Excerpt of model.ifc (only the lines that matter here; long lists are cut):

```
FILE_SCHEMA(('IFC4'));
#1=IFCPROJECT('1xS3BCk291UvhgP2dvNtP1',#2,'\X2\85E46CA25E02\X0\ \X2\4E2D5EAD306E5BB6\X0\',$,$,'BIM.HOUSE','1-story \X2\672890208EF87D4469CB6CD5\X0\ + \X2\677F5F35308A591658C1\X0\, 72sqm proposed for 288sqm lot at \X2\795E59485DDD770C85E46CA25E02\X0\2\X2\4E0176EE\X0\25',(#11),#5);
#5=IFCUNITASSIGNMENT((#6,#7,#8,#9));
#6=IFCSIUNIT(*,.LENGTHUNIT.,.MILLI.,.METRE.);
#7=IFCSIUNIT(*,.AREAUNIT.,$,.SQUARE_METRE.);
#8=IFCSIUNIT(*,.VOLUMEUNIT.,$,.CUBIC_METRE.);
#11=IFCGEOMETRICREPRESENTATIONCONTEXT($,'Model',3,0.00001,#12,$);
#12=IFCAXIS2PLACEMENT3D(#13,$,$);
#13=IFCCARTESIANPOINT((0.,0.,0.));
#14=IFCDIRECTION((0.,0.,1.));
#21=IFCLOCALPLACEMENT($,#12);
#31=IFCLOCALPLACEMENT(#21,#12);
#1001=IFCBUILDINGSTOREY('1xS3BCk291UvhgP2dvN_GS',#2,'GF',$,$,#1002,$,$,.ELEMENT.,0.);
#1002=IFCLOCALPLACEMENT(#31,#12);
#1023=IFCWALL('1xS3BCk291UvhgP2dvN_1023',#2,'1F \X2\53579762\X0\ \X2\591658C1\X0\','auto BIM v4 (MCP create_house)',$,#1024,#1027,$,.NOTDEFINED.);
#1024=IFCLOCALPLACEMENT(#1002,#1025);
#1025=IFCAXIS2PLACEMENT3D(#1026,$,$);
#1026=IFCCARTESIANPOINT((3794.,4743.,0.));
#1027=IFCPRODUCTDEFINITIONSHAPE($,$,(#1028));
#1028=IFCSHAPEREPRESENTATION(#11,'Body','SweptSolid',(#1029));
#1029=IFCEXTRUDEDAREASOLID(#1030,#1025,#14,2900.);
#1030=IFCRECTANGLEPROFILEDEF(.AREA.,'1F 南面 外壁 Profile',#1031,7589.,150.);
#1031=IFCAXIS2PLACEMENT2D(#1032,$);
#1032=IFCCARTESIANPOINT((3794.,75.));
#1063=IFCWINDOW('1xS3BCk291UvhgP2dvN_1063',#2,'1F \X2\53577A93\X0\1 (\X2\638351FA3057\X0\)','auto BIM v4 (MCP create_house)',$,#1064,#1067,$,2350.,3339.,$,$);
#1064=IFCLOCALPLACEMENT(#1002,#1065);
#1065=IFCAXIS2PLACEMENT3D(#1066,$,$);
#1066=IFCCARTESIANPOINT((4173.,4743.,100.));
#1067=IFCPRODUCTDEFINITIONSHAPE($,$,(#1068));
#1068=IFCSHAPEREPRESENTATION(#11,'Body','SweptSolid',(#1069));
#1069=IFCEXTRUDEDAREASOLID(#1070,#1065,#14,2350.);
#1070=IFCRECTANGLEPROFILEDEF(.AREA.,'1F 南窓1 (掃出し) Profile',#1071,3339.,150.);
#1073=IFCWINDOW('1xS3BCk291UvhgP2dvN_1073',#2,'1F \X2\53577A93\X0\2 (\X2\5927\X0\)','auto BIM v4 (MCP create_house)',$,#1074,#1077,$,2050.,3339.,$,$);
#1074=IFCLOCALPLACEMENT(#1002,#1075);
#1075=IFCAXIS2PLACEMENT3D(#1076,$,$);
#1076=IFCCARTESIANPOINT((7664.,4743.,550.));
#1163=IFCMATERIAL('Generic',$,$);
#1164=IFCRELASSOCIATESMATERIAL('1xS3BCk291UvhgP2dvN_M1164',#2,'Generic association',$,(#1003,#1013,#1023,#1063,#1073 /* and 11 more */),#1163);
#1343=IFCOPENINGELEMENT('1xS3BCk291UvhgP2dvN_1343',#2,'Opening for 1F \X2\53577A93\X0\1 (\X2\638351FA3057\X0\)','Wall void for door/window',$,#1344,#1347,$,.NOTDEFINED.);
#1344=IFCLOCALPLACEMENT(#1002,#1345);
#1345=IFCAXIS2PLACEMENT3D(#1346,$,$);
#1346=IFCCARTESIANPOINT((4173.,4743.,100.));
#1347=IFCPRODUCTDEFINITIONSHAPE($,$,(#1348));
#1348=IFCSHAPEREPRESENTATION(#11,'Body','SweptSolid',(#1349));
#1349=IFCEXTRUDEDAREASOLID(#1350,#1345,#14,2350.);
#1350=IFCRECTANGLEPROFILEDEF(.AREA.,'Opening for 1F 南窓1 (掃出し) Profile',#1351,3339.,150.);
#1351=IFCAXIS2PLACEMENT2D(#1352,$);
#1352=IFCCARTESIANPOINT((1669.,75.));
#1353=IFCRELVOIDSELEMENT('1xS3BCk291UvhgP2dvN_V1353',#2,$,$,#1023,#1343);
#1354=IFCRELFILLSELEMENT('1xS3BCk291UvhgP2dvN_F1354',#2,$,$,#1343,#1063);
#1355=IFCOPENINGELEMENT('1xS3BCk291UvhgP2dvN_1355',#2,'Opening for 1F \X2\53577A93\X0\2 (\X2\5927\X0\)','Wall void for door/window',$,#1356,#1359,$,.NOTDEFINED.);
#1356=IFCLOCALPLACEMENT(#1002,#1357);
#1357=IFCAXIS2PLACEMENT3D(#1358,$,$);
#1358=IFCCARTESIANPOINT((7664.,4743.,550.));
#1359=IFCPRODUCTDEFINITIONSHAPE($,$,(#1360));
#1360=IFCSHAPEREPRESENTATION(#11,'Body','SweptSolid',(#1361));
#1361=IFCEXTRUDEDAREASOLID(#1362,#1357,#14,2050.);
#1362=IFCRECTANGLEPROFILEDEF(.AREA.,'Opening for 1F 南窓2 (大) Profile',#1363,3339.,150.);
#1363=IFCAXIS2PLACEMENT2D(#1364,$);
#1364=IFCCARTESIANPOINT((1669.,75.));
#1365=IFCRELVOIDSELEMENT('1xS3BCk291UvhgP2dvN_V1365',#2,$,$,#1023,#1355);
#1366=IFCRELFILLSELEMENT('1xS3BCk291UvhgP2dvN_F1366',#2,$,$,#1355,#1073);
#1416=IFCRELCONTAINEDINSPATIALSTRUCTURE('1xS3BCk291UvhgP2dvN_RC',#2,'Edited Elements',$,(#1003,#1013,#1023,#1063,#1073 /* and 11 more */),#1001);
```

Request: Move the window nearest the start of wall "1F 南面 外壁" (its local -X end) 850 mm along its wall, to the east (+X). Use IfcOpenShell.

```python
import ifcopenshell
import ifcopenshell.api.geometry
import ifcopenshell.util.placement
import ifcopenshell.util.unit

model = ifcopenshell.open("model.ifc")
unit_scale = ifcopenshell.util.unit.calculate_unit_scale(model)

window = model.by_guid("1xS3BCk291UvhgP2dvN_1063")
opening = window.FillsVoids[0].RelatingOpeningElement
wall = opening.VoidsElements[0].RelatingBuildingElement

wall_matrix = ifcopenshell.util.placement.get_local_placement(wall.ObjectPlacement)
shift = wall_matrix[:3, 0] * 0.85 / unit_scale
before = ifcopenshell.util.placement.get_local_placement(window.ObjectPlacement)[:3, 3].copy()

# The window is not placed relative to its opening, so move both.
for product in (opening, window):
    matrix = ifcopenshell.util.placement.get_local_placement(product.ObjectPlacement)
    matrix[:3, 3] += shift
    ifcopenshell.api.geometry.edit_object_placement(model, product=product, matrix=matrix, is_si=False)

after = ifcopenshell.util.placement.get_local_placement(window.ObjectPlacement)[:3, 3]
print("window moved by", (after - before).round(3) + 0.0)

model.write("model_rev.ifc")
```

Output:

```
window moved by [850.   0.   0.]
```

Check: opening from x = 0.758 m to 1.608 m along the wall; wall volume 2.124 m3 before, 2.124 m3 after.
